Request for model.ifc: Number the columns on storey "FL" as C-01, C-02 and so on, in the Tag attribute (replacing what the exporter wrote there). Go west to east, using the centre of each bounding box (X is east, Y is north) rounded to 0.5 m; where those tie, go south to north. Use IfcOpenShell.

First a look at what the model holds.

```python
import ifcopenshell
import ifcopenshell.util.element
import ifcopenshell.util.placement

model = ifcopenshell.open("model.ifc")
print(model.schema)
storey = next(s for s in model.by_type("IfcBuildingStorey") if s.Name == "FL")
columns = [e for e in ifcopenshell.util.element.get_decomposition(storey) if e.is_a("IfcColumn")]
for e in sorted(columns, key=lambda e: e.id()):
    origin = ifcopenshell.util.placement.get_local_placement(e.ObjectPlacement)[:3, 3]
    print(e.id(), e.Tag, e.Name, origin.round(2) + 0.0, sep=" | ")
```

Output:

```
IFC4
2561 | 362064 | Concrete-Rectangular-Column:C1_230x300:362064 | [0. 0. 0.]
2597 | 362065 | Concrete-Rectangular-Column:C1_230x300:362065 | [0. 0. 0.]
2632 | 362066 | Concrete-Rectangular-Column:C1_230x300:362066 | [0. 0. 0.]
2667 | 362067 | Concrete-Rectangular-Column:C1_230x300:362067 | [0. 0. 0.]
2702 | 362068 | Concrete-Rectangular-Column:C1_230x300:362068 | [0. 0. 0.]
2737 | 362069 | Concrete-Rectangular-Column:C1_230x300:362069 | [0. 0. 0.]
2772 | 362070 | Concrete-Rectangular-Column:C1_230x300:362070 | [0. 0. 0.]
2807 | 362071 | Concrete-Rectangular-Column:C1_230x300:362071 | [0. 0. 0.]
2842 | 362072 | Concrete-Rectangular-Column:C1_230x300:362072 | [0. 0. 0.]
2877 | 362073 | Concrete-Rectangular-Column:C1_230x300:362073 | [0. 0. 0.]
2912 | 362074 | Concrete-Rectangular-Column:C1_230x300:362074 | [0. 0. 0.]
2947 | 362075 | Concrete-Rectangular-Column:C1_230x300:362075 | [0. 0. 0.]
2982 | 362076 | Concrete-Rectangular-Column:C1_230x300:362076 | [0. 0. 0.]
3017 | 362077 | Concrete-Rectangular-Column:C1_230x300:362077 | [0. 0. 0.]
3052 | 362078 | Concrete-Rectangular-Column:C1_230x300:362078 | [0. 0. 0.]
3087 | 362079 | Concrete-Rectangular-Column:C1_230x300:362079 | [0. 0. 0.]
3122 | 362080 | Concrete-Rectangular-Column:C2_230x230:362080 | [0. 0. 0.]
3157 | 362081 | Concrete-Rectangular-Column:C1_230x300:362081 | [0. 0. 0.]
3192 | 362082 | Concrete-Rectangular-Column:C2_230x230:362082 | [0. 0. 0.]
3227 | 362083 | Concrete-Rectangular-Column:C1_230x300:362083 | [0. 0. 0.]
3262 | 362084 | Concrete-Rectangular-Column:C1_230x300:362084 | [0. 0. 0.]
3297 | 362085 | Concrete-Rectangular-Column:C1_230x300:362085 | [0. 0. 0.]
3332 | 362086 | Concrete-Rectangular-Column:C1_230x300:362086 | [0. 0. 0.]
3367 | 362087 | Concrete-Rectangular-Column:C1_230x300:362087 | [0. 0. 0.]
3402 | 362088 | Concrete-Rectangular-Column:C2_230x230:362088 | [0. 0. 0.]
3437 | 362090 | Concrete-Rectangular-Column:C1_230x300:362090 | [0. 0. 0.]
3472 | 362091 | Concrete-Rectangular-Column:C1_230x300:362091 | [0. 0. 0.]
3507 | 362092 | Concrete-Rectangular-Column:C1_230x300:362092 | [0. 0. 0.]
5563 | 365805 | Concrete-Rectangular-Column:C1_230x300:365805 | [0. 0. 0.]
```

```python
import ifcopenshell
import ifcopenshell.geom
import ifcopenshell.util.element
import ifcopenshell.util.shape

model = ifcopenshell.open("model.ifc")
settings = ifcopenshell.geom.settings()
settings.set("use-world-coords", True)


def centre(element):
    shape = ifcopenshell.geom.create_shape(settings, element)
    return ifcopenshell.util.shape.get_bbox_centroid(shape.geometry)


storey = next(s for s in model.by_type("IfcBuildingStorey") if s.Name == "FL")
columns = [e for e in ifcopenshell.util.element.get_decomposition(storey) if e.is_a("IfcColumn")]

# Insertion points can sit at a corner or the storey origin, so sort by the geometry (in metres).
centres = {e: centre(e) for e in columns}
columns.sort(key=lambda e: (round(centres[e][0] / 0.5), centres[e][1]))

for i, e in enumerate(columns, start=1):
    number = f"C-{i:02d}"
    e.Tag = number
    print(e.id(), number)

model.write("model_v2.ifc")
```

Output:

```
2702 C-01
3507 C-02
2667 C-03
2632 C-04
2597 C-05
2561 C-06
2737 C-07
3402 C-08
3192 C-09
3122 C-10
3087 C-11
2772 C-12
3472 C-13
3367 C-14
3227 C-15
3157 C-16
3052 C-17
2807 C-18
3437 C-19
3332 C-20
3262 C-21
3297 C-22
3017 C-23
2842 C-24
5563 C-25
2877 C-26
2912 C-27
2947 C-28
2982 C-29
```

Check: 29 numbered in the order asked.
